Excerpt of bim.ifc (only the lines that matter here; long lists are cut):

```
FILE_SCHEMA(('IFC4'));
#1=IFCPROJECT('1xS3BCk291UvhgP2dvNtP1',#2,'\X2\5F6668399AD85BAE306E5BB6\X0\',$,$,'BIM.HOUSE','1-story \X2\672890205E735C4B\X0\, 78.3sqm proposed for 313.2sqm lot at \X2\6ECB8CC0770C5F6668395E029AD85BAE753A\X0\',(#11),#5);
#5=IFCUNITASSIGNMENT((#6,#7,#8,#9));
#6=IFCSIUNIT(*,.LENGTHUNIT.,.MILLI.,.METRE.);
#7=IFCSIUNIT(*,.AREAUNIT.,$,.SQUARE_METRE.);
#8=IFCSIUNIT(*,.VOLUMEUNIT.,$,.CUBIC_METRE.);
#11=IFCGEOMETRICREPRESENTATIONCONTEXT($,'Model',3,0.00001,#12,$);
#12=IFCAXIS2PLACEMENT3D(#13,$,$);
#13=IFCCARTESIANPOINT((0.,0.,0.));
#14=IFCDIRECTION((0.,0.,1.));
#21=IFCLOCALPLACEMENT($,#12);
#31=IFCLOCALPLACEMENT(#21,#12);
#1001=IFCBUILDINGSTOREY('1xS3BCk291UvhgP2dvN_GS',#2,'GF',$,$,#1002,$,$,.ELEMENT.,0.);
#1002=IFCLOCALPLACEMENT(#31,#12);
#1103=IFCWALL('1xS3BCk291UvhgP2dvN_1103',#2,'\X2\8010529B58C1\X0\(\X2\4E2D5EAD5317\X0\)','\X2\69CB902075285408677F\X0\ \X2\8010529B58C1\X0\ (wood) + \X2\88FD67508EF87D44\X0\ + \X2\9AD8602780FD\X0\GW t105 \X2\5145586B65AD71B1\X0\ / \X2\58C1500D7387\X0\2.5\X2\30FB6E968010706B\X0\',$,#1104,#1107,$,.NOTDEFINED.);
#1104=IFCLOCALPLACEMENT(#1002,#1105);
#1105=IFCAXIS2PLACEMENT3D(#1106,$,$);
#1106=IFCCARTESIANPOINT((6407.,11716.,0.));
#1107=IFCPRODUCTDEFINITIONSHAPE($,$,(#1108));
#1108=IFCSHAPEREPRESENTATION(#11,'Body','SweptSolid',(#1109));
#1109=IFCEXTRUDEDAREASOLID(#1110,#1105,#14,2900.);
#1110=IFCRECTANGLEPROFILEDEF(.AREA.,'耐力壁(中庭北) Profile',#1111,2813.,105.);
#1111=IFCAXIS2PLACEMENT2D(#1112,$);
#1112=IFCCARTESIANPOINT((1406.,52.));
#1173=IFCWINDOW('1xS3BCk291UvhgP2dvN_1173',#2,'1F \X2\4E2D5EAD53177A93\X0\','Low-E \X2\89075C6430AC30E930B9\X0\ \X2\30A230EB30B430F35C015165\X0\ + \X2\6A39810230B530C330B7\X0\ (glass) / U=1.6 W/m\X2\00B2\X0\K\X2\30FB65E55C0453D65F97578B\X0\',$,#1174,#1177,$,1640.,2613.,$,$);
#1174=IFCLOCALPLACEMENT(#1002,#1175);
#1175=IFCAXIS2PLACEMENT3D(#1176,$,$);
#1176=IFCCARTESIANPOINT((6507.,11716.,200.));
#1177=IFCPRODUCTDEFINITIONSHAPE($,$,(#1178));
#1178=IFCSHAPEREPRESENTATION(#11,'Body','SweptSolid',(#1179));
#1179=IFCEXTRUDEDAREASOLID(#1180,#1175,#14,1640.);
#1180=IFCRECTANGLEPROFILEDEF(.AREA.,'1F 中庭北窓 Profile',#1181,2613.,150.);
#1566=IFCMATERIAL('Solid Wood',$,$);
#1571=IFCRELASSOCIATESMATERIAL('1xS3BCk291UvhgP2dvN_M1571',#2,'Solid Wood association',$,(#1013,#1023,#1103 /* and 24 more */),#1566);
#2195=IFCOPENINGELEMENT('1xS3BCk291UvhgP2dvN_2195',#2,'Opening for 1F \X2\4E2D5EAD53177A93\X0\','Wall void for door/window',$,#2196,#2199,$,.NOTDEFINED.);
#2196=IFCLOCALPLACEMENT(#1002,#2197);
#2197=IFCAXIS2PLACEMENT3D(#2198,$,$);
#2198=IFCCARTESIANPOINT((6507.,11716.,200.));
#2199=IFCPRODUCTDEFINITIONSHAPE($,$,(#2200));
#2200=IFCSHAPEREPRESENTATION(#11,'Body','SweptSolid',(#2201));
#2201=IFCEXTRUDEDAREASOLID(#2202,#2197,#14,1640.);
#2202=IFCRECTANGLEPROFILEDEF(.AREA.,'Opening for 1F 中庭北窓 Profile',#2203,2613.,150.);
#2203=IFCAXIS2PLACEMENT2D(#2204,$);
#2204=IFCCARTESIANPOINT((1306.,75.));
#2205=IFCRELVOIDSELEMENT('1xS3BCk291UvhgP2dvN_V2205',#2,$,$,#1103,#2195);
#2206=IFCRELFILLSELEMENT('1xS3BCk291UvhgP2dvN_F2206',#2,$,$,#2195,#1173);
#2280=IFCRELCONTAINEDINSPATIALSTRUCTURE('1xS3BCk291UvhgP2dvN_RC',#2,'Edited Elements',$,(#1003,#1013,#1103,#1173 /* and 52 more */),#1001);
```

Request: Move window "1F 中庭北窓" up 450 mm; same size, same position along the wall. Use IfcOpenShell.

```python
import numpy as np
import ifcopenshell
import ifcopenshell.api.geometry
import ifcopenshell.util.placement
import ifcopenshell.util.unit

model = ifcopenshell.open("bim.ifc")
unit_scale = ifcopenshell.util.unit.calculate_unit_scale(model)

window = model.by_guid("1xS3BCk291UvhgP2dvN_1173")
opening = window.FillsVoids[0].RelatingOpeningElement
dz = 0.45 / unit_scale

shift = np.array([0.0, 0.0, dz])
# The window is not placed relative to its opening, so move both.
for product in (opening, window):
    matrix = ifcopenshell.util.placement.get_local_placement(product.ObjectPlacement)
    matrix[:3, 3] += shift
    ifcopenshell.api.geometry.edit_object_placement(model, product=product, matrix=matrix, is_si=False)

print(f"moved by {dz * unit_scale:+.3f} m")

model.write("bim_rev.ifc")
```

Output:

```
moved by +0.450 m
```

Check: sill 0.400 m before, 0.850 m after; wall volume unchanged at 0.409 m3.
